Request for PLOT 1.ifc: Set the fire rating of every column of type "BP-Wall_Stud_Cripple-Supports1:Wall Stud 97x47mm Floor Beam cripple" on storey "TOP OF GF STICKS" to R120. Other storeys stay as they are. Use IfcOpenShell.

First a look at what the model holds.

```python
import ifcopenshell
import ifcopenshell.util.element

model = ifcopenshell.open("PLOT 1.ifc")
print(model.schema)
storey = next(s for s in model.by_type("IfcBuildingStorey") if s.Name == "TOP OF GF STICKS")
columns = [e for e in ifcopenshell.util.element.get_decomposition(storey) if e.is_a("IfcColumn")]
seen = {}
for e in columns:
    element_type = ifcopenshell.util.element.get_type(e)
    key = (element_type.Name if element_type != e and element_type else None, ifcopenshell.util.element.get_pset(e, "Pset_ColumnCommon", "FireRating"))
    seen[key] = seen.get(key, 0) + 1
for (name, value), count in sorted(seen.items(), key=str):
    print(count, "x", name, "|", value)
```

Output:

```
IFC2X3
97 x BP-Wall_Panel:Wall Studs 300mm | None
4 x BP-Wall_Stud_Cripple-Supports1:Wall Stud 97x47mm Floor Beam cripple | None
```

```python
import ifcopenshell
import ifcopenshell.api.pset
import ifcopenshell.util.element

model = ifcopenshell.open("PLOT 1.ifc")

storey = next(s for s in model.by_type("IfcBuildingStorey") if s.Name == "TOP OF GF STICKS")
columns = [e for e in ifcopenshell.util.element.get_decomposition(storey) if e.is_a("IfcColumn")]

count = 0
for e in columns:
    element_type = ifcopenshell.util.element.get_type(e)
    if element_type in (None, e) or element_type.Name != "BP-Wall_Stud_Cripple-Supports1:Wall Stud 97x47mm Floor Beam cripple":
        continue
    # add_pset returns the element's existing set when there is one.
    pset = ifcopenshell.api.pset.add_pset(model, product=e, name="Pset_ColumnCommon")
    ifcopenshell.api.pset.edit_pset(model, pset=pset, properties={"FireRating": "R120"})
    count += 1

print(count, "columns updated")

model.write("PLOT 1_rev.ifc")
```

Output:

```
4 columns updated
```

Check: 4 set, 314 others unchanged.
